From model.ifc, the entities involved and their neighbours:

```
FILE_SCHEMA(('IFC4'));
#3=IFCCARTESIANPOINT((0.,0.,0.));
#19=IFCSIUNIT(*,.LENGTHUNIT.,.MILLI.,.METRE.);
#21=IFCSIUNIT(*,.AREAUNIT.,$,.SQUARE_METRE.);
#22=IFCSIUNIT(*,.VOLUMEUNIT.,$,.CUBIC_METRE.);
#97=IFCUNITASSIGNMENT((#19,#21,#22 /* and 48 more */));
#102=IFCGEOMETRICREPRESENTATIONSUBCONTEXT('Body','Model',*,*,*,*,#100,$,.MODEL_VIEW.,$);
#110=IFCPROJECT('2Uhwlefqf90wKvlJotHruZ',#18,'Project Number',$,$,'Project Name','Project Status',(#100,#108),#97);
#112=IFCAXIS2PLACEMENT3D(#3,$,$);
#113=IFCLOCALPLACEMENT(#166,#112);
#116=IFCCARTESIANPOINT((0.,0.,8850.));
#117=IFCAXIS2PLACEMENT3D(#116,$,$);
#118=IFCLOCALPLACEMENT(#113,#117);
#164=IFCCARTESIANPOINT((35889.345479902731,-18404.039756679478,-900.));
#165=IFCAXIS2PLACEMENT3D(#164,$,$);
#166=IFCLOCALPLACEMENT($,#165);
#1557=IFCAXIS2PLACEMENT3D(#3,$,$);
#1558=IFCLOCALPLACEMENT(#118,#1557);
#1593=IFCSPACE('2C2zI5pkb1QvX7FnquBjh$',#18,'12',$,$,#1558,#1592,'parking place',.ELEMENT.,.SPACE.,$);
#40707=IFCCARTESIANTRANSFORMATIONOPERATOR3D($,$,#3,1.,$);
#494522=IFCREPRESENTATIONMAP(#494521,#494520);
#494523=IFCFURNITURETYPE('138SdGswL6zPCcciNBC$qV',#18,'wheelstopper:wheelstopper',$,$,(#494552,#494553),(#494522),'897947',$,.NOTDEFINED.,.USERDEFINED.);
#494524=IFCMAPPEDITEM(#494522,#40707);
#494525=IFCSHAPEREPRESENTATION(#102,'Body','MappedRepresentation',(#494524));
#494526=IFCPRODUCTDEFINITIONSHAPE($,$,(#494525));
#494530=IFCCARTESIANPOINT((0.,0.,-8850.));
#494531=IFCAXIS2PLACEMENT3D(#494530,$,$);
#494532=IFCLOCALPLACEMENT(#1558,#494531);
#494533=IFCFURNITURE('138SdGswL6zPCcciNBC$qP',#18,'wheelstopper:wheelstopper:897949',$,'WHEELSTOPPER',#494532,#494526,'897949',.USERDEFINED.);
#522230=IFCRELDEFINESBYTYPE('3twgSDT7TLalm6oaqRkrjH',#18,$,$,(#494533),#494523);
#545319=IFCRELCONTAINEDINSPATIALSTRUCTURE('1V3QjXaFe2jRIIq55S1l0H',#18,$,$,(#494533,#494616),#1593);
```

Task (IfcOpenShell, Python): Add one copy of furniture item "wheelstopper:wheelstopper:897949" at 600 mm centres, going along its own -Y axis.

```python
import ifcopenshell
import ifcopenshell.api.geometry
import ifcopenshell.api.root
import ifcopenshell.util.element
import ifcopenshell.util.placement
import ifcopenshell.util.unit

model = ifcopenshell.open("model.ifc")
unit_scale = ifcopenshell.util.unit.calculate_unit_scale(model)


def reuse_history(source, copy):
    """copy_class also copies each property set's owner history, people and application; keep the originals."""
    for rel in copy.IsDefinedBy:
        if rel.is_a("IfcRelDefinesByProperties") and (history := rel.RelatingPropertyDefinition.OwnerHistory):
            rel.RelatingPropertyDefinition.OwnerHistory = source.OwnerHistory
            ifcopenshell.util.element.remove_deep2(model, history)


source = model.by_guid("138SdGswL6zPCcciNBC$qP")
base = ifcopenshell.util.placement.get_local_placement(source.ObjectPlacement)
step = -base[:3, 1] * 0.6 / unit_scale

for i in range(1, 2):
    copy = ifcopenshell.api.root.copy_class(model, product=source)
    copy.Representation = ifcopenshell.util.element.copy_deep(
        model, source.Representation, exclude=["IfcGeometricRepresentationContext", "IfcRepresentationMap"]
    )
    copy.Name = "wheelstopper:wheelstopper"
    copy.Tag = None
    reuse_history(source, copy)
    matrix = base.copy()
    matrix[:3, 3] += i * step
    print("added at", matrix[:3, 3].round(3) + 0.0)
    ifcopenshell.api.geometry.edit_object_placement(model, product=copy, matrix=matrix, is_si=False)

model.write("model_v2.ifc")
```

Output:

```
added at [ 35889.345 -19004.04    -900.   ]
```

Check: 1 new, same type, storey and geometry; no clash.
